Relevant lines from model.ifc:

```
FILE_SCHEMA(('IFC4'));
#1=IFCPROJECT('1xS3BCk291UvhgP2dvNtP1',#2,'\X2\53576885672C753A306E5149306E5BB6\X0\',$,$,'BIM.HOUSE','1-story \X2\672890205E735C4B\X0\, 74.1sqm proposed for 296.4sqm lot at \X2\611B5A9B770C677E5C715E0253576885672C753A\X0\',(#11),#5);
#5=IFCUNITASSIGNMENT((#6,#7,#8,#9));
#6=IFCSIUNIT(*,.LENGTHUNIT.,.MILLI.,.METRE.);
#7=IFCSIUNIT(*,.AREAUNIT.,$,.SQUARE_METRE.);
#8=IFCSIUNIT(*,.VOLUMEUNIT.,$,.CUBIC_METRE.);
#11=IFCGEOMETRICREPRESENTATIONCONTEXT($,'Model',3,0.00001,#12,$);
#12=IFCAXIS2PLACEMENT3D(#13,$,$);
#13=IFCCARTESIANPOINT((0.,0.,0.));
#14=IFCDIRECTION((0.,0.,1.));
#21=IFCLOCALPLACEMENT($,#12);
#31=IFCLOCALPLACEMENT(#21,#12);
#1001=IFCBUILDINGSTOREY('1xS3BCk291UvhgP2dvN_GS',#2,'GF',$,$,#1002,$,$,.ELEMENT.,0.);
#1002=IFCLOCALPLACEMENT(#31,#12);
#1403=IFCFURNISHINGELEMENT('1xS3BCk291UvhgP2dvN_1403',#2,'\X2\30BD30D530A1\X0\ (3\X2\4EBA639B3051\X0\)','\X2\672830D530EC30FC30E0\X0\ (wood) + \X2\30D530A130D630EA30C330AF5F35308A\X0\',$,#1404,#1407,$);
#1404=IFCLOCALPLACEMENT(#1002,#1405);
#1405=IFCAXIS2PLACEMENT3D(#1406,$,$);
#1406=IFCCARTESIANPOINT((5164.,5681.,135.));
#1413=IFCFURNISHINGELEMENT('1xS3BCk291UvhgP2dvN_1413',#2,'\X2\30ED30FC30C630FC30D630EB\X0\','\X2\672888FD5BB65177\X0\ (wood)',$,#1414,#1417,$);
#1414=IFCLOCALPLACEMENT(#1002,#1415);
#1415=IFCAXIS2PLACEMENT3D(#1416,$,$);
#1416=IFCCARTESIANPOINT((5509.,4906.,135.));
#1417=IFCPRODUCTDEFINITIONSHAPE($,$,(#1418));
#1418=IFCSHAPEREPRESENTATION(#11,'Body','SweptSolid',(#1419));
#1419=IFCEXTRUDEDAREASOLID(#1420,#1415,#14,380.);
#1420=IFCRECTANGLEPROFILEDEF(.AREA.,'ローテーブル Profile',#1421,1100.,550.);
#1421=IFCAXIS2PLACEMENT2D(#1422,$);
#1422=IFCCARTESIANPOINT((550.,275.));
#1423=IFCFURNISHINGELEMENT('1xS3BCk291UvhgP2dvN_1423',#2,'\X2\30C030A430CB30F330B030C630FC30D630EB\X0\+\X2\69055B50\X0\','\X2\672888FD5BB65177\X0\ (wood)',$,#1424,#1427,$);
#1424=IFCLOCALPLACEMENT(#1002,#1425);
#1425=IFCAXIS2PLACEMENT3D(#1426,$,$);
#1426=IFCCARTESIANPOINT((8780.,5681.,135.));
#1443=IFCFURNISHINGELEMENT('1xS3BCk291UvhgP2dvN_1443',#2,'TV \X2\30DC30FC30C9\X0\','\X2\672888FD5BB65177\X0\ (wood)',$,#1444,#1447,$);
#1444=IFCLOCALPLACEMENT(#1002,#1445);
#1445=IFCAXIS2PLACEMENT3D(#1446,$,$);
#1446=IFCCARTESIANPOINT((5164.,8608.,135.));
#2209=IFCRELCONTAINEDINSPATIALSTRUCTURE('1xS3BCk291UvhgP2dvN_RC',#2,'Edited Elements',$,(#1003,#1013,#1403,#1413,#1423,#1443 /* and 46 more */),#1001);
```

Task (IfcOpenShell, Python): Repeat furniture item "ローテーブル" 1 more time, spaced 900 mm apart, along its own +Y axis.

```python
import ifcopenshell
import ifcopenshell.api.geometry
import ifcopenshell.api.root
import ifcopenshell.util.element
import ifcopenshell.util.placement
import ifcopenshell.util.unit

model = ifcopenshell.open("model.ifc")
unit_scale = ifcopenshell.util.unit.calculate_unit_scale(model)


def reuse_history(source, copy):
    """copy_class also copies each property set's owner history, people and application; keep the originals."""
    for rel in copy.IsDefinedBy:
        if rel.is_a("IfcRelDefinesByProperties") and (history := rel.RelatingPropertyDefinition.OwnerHistory):
            rel.RelatingPropertyDefinition.OwnerHistory = source.OwnerHistory
            ifcopenshell.util.element.remove_deep2(model, history)


source = model.by_id(1413)
base = ifcopenshell.util.placement.get_local_placement(source.ObjectPlacement)
step = base[:3, 1] * 0.9 / unit_scale

for i in range(1, 2):
    copy = ifcopenshell.api.root.copy_class(model, product=source)
    copy.Representation = ifcopenshell.util.element.copy_deep(
        model, source.Representation, exclude=["IfcGeometricRepresentationContext", "IfcRepresentationMap"]
    )
    reuse_history(source, copy)
    matrix = base.copy()
    matrix[:3, 3] += i * step
    print("added at", matrix[:3, 3].round(3) + 0.0)
    ifcopenshell.api.geometry.edit_object_placement(model, product=copy, matrix=matrix, is_si=False)

model.write("model_v2.ifc")
```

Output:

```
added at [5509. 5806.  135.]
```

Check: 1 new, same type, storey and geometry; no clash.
